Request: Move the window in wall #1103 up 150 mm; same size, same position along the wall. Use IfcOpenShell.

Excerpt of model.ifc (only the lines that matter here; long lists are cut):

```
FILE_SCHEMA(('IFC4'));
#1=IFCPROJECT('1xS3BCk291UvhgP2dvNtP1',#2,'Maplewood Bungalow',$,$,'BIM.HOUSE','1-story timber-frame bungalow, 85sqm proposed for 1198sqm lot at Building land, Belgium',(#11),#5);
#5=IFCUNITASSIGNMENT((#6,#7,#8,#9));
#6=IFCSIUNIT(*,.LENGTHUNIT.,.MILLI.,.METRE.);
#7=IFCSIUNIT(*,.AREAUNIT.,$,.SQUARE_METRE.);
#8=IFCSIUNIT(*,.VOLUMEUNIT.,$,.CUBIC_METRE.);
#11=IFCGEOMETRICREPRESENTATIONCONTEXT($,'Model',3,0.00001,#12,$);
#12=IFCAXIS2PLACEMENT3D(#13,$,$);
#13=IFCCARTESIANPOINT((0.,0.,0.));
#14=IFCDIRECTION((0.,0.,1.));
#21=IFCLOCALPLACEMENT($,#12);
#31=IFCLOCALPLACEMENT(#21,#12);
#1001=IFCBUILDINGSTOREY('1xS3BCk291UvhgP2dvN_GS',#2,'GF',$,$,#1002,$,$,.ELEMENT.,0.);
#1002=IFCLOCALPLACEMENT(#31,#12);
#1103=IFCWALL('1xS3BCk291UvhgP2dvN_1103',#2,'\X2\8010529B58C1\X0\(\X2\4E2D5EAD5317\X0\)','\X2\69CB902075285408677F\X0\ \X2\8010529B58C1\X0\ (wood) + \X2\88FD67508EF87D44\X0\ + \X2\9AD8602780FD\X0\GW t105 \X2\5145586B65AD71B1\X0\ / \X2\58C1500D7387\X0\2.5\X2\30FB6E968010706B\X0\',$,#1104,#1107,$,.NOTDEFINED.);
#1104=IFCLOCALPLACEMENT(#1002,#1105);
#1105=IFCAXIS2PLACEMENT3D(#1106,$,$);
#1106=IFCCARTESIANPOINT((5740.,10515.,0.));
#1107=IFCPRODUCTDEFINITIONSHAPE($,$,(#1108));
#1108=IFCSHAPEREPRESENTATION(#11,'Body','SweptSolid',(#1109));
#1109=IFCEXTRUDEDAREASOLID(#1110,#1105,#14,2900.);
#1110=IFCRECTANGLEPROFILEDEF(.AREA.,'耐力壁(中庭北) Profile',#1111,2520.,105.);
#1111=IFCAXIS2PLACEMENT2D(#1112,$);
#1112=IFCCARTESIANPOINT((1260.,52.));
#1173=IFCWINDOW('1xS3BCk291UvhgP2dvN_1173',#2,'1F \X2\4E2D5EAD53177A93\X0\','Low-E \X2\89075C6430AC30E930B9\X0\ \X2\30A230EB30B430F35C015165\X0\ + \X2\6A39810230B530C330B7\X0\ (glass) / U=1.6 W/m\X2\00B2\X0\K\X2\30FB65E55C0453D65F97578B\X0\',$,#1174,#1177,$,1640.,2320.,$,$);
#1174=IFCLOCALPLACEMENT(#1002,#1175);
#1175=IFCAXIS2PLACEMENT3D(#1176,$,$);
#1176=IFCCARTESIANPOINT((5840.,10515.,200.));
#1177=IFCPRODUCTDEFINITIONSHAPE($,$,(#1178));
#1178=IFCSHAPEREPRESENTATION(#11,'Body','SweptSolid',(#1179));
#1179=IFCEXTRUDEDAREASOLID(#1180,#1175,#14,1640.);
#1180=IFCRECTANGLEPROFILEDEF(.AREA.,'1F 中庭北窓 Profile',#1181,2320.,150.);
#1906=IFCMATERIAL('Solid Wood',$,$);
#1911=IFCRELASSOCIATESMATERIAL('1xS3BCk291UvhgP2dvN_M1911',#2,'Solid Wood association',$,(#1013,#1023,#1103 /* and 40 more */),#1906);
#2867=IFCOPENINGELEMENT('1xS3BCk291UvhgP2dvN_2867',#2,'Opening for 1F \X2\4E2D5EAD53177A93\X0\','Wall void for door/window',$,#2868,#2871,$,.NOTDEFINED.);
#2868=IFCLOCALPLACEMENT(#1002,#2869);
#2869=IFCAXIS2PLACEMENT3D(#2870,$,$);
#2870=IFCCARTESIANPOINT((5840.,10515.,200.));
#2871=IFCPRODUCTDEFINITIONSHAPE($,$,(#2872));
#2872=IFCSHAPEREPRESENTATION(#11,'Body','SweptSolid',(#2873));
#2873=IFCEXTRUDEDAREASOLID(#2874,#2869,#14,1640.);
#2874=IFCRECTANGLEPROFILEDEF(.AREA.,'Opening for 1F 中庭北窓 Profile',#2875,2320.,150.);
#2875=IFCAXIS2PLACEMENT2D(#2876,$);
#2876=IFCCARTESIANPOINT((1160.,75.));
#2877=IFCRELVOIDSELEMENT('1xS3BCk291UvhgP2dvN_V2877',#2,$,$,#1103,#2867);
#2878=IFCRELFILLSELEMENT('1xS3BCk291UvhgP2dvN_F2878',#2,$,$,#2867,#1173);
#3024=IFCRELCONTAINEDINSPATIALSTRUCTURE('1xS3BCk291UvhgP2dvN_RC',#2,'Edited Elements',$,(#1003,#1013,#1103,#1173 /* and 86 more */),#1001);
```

```python
import numpy as np
import ifcopenshell
import ifcopenshell.api.geometry
import ifcopenshell.util.placement
import ifcopenshell.util.unit

model = ifcopenshell.open("model.ifc")
unit_scale = ifcopenshell.util.unit.calculate_unit_scale(model)

window = model.by_guid("1xS3BCk291UvhgP2dvN_1173")
opening = window.FillsVoids[0].RelatingOpeningElement
dz = 0.15 / unit_scale

shift = np.array([0.0, 0.0, dz])
# The window is not placed relative to its opening, so move both.
for product in (opening, window):
    matrix = ifcopenshell.util.placement.get_local_placement(product.ObjectPlacement)
    matrix[:3, 3] += shift
    ifcopenshell.api.geometry.edit_object_placement(model, product=product, matrix=matrix, is_si=False)

print(f"moved by {dz * unit_scale:+.3f} m")

model.write("model_edited.ifc")
```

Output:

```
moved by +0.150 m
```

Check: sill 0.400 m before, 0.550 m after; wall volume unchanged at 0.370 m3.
